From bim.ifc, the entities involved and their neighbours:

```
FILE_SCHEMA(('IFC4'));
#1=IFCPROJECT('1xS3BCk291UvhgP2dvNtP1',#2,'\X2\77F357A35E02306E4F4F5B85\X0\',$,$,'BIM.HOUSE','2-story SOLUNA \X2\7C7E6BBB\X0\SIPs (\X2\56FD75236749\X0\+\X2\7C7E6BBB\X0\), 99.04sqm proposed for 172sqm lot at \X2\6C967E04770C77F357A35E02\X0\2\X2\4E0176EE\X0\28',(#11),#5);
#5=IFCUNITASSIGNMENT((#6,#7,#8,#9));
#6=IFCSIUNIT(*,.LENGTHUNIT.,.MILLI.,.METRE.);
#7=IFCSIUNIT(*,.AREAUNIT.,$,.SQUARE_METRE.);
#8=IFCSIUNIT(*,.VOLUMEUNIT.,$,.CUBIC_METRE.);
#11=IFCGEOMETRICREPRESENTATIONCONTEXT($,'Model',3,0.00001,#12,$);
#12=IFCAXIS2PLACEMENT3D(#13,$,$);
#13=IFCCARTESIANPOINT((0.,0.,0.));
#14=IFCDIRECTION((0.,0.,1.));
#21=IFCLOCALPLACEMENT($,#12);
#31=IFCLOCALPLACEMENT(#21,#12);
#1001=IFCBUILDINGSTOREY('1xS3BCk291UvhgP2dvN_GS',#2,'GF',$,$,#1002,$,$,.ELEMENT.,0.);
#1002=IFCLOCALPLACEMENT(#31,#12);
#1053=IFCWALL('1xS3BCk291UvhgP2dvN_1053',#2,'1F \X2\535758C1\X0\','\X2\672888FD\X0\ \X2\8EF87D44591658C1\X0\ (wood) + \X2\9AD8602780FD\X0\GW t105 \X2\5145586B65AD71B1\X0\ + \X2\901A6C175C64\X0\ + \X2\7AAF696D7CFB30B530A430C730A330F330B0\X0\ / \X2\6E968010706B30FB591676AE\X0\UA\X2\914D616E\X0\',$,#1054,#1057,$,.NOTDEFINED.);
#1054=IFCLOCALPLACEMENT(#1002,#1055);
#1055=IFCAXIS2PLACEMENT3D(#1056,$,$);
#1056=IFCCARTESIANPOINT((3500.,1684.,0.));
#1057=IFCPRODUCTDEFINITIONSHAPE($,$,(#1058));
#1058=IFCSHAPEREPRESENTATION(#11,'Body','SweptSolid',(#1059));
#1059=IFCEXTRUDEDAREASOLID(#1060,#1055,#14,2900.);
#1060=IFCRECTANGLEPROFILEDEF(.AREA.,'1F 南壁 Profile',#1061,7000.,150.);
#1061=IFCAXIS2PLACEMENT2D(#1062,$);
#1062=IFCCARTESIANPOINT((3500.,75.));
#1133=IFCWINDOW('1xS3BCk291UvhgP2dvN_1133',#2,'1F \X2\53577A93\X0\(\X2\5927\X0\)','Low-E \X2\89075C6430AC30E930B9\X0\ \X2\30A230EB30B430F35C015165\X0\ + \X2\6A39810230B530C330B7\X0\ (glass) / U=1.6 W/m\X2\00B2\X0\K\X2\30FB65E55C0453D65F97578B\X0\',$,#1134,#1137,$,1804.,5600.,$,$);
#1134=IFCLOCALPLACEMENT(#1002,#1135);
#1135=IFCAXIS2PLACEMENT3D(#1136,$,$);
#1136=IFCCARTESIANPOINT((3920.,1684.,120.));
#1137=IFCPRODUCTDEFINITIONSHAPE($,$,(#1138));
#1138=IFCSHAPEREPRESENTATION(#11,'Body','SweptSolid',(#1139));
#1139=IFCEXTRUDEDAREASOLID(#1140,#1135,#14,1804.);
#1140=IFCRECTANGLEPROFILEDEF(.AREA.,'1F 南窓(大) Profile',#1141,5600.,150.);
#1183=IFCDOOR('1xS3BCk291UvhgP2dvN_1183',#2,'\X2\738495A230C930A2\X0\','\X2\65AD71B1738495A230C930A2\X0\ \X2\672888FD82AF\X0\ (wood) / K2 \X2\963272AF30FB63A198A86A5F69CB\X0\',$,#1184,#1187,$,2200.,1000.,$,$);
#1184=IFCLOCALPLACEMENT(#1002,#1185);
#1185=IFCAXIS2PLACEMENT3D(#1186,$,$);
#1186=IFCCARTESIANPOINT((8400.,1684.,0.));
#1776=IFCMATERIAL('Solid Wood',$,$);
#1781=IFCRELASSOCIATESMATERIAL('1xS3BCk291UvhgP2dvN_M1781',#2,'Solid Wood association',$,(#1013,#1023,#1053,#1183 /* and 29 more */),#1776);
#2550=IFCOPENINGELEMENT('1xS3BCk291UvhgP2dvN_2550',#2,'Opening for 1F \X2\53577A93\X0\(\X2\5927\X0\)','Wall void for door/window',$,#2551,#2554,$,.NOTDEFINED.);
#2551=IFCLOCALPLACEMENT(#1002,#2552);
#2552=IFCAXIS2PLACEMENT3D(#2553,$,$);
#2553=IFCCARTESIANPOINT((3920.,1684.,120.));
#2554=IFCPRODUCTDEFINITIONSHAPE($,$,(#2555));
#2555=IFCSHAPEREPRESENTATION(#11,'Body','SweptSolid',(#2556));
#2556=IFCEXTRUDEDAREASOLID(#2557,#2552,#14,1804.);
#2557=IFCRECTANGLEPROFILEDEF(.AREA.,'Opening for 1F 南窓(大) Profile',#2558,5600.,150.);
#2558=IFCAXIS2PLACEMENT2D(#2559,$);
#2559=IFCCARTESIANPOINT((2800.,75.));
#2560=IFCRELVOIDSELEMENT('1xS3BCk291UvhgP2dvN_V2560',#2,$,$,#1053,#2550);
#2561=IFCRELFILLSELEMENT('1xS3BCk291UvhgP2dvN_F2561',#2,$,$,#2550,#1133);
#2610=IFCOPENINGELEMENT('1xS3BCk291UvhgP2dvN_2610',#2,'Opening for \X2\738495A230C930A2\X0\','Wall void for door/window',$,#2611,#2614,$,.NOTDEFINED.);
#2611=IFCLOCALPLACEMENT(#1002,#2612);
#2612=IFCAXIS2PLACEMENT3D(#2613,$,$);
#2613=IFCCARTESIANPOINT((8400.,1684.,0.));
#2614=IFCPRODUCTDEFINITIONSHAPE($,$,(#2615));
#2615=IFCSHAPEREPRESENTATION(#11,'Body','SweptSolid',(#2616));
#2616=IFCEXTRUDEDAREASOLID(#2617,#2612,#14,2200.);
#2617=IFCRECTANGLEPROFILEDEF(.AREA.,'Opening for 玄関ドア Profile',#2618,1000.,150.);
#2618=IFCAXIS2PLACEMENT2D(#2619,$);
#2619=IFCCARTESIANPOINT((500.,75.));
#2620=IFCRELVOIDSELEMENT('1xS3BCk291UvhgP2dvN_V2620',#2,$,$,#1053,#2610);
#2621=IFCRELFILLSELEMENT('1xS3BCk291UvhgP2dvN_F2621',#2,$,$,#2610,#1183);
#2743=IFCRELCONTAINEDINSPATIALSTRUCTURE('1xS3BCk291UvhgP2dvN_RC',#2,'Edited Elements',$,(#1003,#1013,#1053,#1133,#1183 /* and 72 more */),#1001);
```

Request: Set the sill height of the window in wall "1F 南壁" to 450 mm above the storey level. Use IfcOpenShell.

```python
import numpy as np
import ifcopenshell
import ifcopenshell.api.geometry
import ifcopenshell.geom
import ifcopenshell.util.element
import ifcopenshell.util.placement
import ifcopenshell.util.shape
import ifcopenshell.util.unit

model = ifcopenshell.open("bim.ifc")
unit_scale = ifcopenshell.util.unit.calculate_unit_scale(model)

window = model.by_id(1133)
opening = window.FillsVoids[0].RelatingOpeningElement
storey = ifcopenshell.util.element.get_container(window, ifc_class="IfcBuildingStorey")
level = ifcopenshell.util.placement.get_local_placement(storey.ObjectPlacement)[2, 3]

# The opening's origin need not be at the sill, so measure its lowest point.
shape = ifcopenshell.geom.create_shape(ifcopenshell.geom.settings(), opening)
bottom = ifcopenshell.util.shape.get_shape_bottom_elevation(shape, shape.geometry) / unit_scale
dz = level + 0.45 / unit_scale - bottom

shift = np.array([0.0, 0.0, dz])
# The window is not placed relative to its opening, so move both.
for product in (opening, window):
    matrix = ifcopenshell.util.placement.get_local_placement(product.ObjectPlacement)
    matrix[:3, 3] += shift
    ifcopenshell.api.geometry.edit_object_placement(model, product=product, matrix=matrix, is_si=False)

print(f"moved by {dz * unit_scale:+.3f} m")

model.write("bim_edited.ifc")
```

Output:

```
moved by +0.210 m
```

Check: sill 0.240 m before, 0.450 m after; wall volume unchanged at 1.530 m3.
